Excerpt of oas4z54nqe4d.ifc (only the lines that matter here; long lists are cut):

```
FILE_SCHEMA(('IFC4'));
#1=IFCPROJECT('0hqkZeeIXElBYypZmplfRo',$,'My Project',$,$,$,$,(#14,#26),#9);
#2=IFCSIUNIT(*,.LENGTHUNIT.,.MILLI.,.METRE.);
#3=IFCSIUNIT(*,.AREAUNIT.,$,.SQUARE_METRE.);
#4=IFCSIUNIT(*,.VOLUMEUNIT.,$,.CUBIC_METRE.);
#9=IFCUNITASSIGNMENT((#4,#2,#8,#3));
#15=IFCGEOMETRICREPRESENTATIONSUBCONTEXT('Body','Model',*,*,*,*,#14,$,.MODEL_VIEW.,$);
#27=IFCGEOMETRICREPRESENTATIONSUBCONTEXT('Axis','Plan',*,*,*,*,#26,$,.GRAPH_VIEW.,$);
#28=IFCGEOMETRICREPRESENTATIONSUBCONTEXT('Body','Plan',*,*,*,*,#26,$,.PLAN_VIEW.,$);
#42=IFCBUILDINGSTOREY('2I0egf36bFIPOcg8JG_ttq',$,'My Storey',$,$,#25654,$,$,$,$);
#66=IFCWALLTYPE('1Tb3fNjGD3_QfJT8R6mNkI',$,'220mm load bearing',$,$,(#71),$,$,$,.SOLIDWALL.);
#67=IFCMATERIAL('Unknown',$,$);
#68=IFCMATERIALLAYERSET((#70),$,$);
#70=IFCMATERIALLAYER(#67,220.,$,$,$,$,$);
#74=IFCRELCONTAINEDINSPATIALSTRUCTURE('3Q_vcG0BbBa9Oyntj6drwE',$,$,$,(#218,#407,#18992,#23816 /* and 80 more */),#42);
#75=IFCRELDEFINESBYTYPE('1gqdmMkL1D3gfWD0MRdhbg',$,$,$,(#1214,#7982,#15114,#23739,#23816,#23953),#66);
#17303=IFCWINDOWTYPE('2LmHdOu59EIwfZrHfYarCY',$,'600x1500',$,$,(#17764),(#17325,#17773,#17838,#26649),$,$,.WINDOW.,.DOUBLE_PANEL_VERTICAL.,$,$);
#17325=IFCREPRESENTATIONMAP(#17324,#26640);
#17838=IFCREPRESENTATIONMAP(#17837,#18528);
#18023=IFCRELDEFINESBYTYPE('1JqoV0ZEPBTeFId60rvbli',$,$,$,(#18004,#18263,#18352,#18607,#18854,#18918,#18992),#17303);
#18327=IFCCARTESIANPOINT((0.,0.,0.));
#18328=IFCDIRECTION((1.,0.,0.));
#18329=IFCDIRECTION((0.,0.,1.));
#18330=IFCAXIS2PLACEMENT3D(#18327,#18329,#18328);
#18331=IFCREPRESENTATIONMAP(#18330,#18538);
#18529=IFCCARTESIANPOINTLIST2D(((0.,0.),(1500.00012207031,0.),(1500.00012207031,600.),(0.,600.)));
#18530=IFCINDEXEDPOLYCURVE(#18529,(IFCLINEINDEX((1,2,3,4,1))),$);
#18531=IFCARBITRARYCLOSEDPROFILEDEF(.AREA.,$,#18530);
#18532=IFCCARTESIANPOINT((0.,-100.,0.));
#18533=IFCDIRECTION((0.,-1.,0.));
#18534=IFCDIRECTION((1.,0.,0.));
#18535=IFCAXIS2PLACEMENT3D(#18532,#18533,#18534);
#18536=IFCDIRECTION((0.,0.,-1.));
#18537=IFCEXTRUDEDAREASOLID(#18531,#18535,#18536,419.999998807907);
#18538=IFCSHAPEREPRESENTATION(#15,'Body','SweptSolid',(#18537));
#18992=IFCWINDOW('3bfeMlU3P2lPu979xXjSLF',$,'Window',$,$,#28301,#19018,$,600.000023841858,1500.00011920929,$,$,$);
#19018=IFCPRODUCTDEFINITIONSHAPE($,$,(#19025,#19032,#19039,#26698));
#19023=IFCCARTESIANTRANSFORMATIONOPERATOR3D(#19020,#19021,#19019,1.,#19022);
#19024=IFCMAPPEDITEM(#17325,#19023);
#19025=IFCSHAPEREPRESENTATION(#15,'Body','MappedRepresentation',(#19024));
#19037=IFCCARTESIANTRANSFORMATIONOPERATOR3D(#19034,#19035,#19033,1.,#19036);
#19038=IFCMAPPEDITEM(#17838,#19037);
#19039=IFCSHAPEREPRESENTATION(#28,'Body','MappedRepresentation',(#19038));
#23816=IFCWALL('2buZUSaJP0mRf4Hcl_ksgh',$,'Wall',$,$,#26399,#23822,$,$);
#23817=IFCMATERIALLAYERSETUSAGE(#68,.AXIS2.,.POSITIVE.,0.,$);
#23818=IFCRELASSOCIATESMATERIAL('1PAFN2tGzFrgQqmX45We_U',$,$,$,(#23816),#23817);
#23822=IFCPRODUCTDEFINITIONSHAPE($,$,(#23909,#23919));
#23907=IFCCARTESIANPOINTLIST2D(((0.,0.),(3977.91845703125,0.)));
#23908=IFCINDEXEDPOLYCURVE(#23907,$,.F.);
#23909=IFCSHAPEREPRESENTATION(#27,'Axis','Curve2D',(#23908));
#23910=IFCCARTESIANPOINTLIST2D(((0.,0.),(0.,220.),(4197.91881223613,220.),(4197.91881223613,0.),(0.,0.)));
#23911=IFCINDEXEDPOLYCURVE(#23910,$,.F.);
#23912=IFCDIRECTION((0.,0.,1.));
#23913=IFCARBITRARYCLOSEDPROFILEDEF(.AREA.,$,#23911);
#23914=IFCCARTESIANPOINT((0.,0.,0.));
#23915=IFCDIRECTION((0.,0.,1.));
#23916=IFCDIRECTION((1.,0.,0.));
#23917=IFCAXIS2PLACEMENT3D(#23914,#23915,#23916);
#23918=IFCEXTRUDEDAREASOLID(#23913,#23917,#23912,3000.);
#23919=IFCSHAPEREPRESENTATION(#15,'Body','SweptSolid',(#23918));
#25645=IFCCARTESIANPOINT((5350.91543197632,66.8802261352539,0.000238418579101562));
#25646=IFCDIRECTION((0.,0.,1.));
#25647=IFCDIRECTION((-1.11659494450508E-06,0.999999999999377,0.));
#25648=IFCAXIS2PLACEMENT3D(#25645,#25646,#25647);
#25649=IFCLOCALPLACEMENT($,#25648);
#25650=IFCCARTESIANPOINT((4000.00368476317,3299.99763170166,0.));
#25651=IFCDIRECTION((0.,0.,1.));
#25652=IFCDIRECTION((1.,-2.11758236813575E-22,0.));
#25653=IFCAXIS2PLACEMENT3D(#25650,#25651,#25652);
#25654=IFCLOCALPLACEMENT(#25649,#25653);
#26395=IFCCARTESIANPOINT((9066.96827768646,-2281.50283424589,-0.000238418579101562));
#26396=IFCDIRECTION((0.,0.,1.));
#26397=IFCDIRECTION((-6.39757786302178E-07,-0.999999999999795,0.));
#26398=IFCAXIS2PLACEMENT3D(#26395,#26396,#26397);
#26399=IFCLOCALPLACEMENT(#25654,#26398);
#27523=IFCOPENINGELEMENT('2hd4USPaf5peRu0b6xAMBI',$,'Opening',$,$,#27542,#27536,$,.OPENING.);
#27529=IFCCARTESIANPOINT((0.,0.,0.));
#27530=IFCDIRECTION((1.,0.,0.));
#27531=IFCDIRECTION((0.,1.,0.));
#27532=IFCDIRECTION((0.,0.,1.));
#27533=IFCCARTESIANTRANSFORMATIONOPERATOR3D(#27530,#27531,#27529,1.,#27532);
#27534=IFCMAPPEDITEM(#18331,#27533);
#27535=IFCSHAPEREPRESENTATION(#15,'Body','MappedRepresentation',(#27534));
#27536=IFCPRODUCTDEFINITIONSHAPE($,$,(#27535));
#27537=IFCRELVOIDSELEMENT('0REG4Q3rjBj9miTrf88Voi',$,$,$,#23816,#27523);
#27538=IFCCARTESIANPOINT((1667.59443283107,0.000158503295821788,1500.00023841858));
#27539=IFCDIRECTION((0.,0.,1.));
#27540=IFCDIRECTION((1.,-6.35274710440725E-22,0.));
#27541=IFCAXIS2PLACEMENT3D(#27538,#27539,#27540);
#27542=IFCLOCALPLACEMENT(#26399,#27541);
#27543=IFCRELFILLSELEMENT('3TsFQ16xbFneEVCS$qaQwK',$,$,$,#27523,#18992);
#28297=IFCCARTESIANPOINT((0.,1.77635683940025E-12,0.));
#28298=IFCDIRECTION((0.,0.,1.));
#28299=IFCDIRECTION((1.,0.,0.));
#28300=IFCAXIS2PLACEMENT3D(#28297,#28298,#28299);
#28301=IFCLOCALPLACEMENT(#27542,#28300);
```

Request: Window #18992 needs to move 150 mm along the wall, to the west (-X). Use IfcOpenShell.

```python
import ifcopenshell
import ifcopenshell.api.geometry
import ifcopenshell.util.placement
import ifcopenshell.util.unit

model = ifcopenshell.open("oas4z54nqe4d.ifc")
unit_scale = ifcopenshell.util.unit.calculate_unit_scale(model)

window = model.by_guid("3bfeMlU3P2lPu979xXjSLF")
opening = window.FillsVoids[0].RelatingOpeningElement
wall = opening.VoidsElements[0].RelatingBuildingElement

wall_matrix = ifcopenshell.util.placement.get_local_placement(wall.ObjectPlacement)
shift = wall_matrix[:3, 0] * -0.15 / unit_scale
before = ifcopenshell.util.placement.get_local_placement(window.ObjectPlacement)[:3, 3].copy()

# The window is placed relative to its opening, so it follows when the opening moves.
matrix = ifcopenshell.util.placement.get_local_placement(opening.ObjectPlacement)
matrix[:3, 3] += shift
ifcopenshell.api.geometry.edit_object_placement(
    model, product=opening, matrix=matrix, is_si=False, should_transform_children=True
)

after = ifcopenshell.util.placement.get_local_placement(window.ObjectPlacement)[:3, 3]
print("window moved by", (after - before).round(3) + 0.0)

model.write("oas4z54nqe4d_v2.ifc")
```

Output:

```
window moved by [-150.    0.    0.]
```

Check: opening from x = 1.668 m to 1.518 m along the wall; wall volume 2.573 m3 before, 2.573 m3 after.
